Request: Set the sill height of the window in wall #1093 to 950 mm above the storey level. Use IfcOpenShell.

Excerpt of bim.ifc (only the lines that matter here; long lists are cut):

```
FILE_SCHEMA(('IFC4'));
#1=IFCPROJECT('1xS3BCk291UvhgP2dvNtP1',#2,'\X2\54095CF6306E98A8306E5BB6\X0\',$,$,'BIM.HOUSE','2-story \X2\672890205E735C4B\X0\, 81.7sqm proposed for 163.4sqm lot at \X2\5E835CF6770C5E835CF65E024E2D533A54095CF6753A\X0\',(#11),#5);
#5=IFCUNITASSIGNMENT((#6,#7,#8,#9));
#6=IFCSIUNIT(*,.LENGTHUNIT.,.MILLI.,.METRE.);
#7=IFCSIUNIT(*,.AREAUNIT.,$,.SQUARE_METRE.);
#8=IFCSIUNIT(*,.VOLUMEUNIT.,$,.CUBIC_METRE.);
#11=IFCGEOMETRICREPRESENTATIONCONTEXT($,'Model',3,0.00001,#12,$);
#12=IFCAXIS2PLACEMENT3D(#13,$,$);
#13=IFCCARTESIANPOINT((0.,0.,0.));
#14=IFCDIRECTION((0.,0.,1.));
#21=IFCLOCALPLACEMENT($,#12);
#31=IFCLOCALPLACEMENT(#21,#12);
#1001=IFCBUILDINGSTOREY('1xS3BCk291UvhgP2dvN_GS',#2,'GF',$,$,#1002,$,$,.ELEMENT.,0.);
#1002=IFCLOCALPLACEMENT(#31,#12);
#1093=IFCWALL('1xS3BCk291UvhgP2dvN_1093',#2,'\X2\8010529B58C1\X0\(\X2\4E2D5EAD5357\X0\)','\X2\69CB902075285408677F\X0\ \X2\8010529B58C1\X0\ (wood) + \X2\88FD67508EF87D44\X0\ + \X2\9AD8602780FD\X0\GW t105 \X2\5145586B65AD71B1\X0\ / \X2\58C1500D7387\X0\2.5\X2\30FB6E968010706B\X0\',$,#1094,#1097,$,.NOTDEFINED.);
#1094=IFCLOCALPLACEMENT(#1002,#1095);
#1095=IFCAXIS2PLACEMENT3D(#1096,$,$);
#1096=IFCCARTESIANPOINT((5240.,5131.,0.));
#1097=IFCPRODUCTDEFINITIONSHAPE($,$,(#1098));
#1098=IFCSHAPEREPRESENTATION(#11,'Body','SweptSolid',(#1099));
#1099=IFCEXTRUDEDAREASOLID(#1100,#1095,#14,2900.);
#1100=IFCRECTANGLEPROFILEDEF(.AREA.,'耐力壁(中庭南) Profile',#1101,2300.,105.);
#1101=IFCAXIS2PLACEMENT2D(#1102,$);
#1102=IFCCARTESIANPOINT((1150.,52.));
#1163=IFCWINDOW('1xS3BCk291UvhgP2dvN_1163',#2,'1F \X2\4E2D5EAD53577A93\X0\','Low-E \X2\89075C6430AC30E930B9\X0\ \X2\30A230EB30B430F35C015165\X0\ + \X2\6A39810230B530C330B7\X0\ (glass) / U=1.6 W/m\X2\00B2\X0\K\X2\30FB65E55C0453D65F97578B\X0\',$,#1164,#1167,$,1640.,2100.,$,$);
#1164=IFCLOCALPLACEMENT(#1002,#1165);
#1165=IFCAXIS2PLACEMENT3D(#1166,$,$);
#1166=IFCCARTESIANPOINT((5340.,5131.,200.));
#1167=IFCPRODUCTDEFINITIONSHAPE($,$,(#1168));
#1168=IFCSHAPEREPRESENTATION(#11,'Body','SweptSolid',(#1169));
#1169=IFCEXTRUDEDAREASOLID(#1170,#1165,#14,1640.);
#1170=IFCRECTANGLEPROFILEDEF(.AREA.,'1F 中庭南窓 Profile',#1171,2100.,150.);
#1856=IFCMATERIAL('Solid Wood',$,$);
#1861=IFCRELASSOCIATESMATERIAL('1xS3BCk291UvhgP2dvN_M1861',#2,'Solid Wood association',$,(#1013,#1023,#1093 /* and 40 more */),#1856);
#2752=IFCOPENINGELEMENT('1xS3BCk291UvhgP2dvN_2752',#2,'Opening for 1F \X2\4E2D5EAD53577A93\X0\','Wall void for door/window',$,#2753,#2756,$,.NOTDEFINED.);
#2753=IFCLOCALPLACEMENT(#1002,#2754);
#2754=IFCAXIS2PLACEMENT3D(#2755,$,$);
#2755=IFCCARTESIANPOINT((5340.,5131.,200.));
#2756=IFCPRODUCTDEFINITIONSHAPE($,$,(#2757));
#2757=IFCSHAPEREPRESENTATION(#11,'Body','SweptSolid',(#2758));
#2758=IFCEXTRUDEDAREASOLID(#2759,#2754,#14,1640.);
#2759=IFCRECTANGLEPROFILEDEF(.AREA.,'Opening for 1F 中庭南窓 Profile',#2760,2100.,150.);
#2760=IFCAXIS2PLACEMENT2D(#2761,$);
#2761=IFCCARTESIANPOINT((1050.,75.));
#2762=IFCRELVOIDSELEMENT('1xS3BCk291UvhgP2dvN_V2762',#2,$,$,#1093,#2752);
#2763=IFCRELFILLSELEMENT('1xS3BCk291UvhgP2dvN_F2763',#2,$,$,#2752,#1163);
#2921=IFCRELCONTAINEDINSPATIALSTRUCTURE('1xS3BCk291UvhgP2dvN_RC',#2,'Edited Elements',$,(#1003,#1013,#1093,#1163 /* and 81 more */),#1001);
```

```python
import numpy as np
import ifcopenshell
import ifcopenshell.api.geometry
import ifcopenshell.geom
import ifcopenshell.util.element
import ifcopenshell.util.placement
import ifcopenshell.util.shape
import ifcopenshell.util.unit

model = ifcopenshell.open("bim.ifc")
unit_scale = ifcopenshell.util.unit.calculate_unit_scale(model)

window = model.by_guid("1xS3BCk291UvhgP2dvN_1163")
opening = window.FillsVoids[0].RelatingOpeningElement
storey = ifcopenshell.util.element.get_container(window, ifc_class="IfcBuildingStorey")
level = ifcopenshell.util.placement.get_local_placement(storey.ObjectPlacement)[2, 3]

# The opening's origin need not be at the sill, so measure its lowest point.
shape = ifcopenshell.geom.create_shape(ifcopenshell.geom.settings(), opening)
bottom = ifcopenshell.util.shape.get_shape_bottom_elevation(shape, shape.geometry) / unit_scale
dz = level + 0.95 / unit_scale - bottom

shift = np.array([0.0, 0.0, dz])
# The window is not placed relative to its opening, so move both.
for product in (opening, window):
    matrix = ifcopenshell.util.placement.get_local_placement(product.ObjectPlacement)
    matrix[:3, 3] += shift
    ifcopenshell.api.geometry.edit_object_placement(model, product=product, matrix=matrix, is_si=False)

print(f"moved by {dz * unit_scale:+.3f} m")

model.write("bim_v2.ifc")
```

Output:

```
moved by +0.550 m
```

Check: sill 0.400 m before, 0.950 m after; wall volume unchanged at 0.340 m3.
